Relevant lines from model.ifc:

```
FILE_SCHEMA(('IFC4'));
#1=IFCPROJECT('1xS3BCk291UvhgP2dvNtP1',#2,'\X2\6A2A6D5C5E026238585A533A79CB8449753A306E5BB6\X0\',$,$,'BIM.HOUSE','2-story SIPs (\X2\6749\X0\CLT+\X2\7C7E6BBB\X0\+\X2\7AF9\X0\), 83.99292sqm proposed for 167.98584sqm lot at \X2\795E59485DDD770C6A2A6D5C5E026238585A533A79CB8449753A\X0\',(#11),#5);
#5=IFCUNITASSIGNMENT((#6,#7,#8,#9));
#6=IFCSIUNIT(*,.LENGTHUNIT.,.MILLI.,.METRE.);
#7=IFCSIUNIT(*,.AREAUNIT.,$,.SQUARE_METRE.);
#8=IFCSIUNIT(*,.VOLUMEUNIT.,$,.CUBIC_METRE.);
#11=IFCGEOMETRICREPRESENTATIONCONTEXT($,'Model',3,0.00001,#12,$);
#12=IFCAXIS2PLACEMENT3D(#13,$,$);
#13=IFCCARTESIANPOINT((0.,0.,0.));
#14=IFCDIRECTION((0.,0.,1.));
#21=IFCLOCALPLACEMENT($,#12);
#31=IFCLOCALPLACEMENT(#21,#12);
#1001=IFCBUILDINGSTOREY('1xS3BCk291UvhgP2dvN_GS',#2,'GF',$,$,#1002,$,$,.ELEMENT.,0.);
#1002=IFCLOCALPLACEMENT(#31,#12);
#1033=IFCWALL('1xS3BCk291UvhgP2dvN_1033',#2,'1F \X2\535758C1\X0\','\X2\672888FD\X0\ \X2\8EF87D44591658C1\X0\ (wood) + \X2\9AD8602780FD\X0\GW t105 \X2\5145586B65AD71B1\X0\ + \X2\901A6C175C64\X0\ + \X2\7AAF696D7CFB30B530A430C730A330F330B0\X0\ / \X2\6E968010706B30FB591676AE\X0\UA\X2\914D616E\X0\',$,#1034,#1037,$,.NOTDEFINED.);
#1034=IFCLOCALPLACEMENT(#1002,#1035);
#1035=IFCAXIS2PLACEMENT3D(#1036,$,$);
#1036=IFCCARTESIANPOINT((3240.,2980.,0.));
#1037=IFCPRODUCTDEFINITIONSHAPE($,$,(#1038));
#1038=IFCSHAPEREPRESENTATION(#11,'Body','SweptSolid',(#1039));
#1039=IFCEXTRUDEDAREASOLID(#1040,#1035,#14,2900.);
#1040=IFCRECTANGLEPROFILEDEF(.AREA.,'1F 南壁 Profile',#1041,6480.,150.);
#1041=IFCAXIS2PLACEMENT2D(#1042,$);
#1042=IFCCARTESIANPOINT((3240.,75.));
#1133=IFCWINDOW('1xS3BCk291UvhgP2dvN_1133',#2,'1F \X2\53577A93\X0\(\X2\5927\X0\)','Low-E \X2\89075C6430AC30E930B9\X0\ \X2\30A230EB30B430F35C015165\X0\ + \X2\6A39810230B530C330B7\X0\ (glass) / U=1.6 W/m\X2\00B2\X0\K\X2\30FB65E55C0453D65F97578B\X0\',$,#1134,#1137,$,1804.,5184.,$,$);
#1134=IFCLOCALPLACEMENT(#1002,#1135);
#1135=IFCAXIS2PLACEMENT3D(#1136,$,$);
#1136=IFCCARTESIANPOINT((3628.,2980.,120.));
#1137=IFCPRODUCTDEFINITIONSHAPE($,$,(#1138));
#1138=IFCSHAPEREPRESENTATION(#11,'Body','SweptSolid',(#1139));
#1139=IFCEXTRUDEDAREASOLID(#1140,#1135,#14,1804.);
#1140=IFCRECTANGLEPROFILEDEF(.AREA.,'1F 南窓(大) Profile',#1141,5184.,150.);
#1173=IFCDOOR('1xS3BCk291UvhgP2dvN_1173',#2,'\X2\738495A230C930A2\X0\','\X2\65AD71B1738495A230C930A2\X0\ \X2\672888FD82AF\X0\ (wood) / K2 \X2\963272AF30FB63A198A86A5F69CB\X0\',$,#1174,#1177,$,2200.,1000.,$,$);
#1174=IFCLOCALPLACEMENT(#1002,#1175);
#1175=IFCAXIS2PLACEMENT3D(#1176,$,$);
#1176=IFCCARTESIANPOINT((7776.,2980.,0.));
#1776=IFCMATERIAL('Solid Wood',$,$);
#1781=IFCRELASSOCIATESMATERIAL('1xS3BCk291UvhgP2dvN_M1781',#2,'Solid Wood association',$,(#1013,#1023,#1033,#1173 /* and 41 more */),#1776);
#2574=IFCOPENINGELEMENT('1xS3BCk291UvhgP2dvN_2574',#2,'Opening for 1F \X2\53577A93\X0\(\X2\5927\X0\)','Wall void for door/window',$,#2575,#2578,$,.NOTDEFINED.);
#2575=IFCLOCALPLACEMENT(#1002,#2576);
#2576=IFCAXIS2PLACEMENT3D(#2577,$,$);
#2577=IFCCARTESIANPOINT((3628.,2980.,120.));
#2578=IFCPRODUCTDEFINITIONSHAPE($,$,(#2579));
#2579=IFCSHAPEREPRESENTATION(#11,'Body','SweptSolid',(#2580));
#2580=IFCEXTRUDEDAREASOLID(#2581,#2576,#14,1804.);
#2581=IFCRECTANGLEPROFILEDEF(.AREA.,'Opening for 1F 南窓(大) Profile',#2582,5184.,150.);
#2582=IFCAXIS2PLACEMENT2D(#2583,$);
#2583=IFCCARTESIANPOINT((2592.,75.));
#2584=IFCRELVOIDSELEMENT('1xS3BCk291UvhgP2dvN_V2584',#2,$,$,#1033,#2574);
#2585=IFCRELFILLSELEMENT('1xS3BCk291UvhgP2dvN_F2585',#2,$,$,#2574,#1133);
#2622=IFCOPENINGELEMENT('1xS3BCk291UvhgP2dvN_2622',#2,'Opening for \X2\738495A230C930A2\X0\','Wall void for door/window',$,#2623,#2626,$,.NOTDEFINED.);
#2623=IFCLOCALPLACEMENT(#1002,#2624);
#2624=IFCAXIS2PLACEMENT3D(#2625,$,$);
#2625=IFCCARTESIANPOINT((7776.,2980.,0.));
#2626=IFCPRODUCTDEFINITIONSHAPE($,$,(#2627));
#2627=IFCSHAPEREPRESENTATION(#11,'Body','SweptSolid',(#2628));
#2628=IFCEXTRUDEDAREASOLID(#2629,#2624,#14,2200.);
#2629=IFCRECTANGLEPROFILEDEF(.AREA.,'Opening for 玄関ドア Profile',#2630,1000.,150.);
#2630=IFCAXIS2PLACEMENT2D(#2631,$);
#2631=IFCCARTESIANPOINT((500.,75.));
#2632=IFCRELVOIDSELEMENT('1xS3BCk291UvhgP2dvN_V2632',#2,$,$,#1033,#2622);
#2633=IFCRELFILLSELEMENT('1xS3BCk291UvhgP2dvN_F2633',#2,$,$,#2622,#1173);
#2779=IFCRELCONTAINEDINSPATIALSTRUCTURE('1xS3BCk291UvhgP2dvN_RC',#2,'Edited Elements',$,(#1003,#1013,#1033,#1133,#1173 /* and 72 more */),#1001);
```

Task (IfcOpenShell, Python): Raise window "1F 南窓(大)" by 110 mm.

```python
import numpy as np
import ifcopenshell
import ifcopenshell.api.geometry
import ifcopenshell.util.placement
import ifcopenshell.util.unit

model = ifcopenshell.open("model.ifc")
unit_scale = ifcopenshell.util.unit.calculate_unit_scale(model)

window = model.by_guid("1xS3BCk291UvhgP2dvN_1133")
opening = window.FillsVoids[0].RelatingOpeningElement
dz = 110.0

shift = np.array([0.0, 0.0, dz])
# The window is not placed relative to its opening, so move both.
for product in (opening, window):
    matrix = ifcopenshell.util.placement.get_local_placement(product.ObjectPlacement)
    matrix[:3, 3] += shift
    ifcopenshell.api.geometry.edit_object_placement(model, product=product, matrix=matrix, is_si=False)

print(f"moved by {dz * unit_scale:+.3f} m")

model.write("model_v2.ifc")
```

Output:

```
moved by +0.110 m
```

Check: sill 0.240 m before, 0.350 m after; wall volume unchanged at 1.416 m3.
